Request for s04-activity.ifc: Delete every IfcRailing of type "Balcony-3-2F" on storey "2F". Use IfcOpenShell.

First a look at what the model holds.

```python
import ifcopenshell
import ifcopenshell.util.element

model = ifcopenshell.open("s04-activity.ifc")
print(model.schema)
storey = next(s for s in model.by_type("IfcBuildingStorey") if s.Name == "2F")
railings = [e for e in ifcopenshell.util.element.get_decomposition(storey) if e.is_a("IfcRailing")]
seen = {}
for e in railings:
    element_type = ifcopenshell.util.element.get_type(e)
    name = element_type.Name if element_type not in (None, e) else None
    seen[name] = seen.get(name, 0) + 1
for name, count in sorted(seen.items(), key=str):
    print(count, "x", name)
```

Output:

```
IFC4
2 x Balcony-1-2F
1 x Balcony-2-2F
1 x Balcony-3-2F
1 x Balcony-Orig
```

```python
import ifcopenshell
import ifcopenshell.api.root
import ifcopenshell.util.element

model = ifcopenshell.open("s04-activity.ifc")

storey = next(s for s in model.by_type("IfcBuildingStorey") if s.Name == "2F")
railings = [e for e in ifcopenshell.util.element.get_decomposition(storey) if e.is_a("IfcRailing")]
targets = [e for e in railings if (t := ifcopenshell.util.element.get_type(e)) not in (None, e) and t.Name == "Balcony-3-2F"]

for e in targets:
    ifcopenshell.api.root.remove_product(model, product=e)
print(len(targets), "removed")

model.write("s04-activity_v2.ifc")
```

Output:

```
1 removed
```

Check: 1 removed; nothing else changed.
